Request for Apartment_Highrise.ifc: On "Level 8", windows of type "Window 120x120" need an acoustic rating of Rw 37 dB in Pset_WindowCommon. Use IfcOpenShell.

First a look at what the model holds.

```python
import ifcopenshell
import ifcopenshell.util.element

model = ifcopenshell.open("Apartment_Highrise.ifc")
print(model.schema)
storey = next(s for s in model.by_type("IfcBuildingStorey") if s.Name == "Level 8")
windows = [e for e in ifcopenshell.util.element.get_decomposition(storey) if e.is_a("IfcWindow")]
seen = {}
for e in windows:
    element_type = ifcopenshell.util.element.get_type(e)
    key = (element_type.Name if element_type != e and element_type else None, ifcopenshell.util.element.get_pset(e, "Pset_WindowCommon", "AcousticRating"))
    seen[key] = seen.get(key, 0) + 1
for (name, value), count in sorted(seen.items(), key=str):
    print(count, "x", name, "|", value)
```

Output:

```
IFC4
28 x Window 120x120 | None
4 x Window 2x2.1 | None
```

```python
import ifcopenshell
import ifcopenshell.api.pset
import ifcopenshell.util.element

model = ifcopenshell.open("Apartment_Highrise.ifc")

storey = next(s for s in model.by_type("IfcBuildingStorey") if s.Name == "Level 8")
windows = [e for e in ifcopenshell.util.element.get_decomposition(storey) if e.is_a("IfcWindow")]

count = 0
for e in windows:
    element_type = ifcopenshell.util.element.get_type(e)
    if element_type in (None, e) or element_type.Name != "Window 120x120":
        continue
    found = ifcopenshell.util.element.get_pset(e, "Pset_WindowCommon", should_inherit=False)
    if found:
        pset = model.by_id(found["id"])
        if len(ifcopenshell.util.element.get_elements_by_pset(pset)) > 1:
            pset = ifcopenshell.api.pset.unshare_pset(model, products=[e], pset=pset)[0]
    else:
        pset = ifcopenshell.api.pset.add_pset(model, product=e, name="Pset_WindowCommon")
    ifcopenshell.api.pset.edit_pset(model, pset=pset, properties={"AcousticRating": "Rw 37 dB"})
    count += 1

print(count, "windows updated")

model.write("Apartment_Highrise_edited.ifc")
```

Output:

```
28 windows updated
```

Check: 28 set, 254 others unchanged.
